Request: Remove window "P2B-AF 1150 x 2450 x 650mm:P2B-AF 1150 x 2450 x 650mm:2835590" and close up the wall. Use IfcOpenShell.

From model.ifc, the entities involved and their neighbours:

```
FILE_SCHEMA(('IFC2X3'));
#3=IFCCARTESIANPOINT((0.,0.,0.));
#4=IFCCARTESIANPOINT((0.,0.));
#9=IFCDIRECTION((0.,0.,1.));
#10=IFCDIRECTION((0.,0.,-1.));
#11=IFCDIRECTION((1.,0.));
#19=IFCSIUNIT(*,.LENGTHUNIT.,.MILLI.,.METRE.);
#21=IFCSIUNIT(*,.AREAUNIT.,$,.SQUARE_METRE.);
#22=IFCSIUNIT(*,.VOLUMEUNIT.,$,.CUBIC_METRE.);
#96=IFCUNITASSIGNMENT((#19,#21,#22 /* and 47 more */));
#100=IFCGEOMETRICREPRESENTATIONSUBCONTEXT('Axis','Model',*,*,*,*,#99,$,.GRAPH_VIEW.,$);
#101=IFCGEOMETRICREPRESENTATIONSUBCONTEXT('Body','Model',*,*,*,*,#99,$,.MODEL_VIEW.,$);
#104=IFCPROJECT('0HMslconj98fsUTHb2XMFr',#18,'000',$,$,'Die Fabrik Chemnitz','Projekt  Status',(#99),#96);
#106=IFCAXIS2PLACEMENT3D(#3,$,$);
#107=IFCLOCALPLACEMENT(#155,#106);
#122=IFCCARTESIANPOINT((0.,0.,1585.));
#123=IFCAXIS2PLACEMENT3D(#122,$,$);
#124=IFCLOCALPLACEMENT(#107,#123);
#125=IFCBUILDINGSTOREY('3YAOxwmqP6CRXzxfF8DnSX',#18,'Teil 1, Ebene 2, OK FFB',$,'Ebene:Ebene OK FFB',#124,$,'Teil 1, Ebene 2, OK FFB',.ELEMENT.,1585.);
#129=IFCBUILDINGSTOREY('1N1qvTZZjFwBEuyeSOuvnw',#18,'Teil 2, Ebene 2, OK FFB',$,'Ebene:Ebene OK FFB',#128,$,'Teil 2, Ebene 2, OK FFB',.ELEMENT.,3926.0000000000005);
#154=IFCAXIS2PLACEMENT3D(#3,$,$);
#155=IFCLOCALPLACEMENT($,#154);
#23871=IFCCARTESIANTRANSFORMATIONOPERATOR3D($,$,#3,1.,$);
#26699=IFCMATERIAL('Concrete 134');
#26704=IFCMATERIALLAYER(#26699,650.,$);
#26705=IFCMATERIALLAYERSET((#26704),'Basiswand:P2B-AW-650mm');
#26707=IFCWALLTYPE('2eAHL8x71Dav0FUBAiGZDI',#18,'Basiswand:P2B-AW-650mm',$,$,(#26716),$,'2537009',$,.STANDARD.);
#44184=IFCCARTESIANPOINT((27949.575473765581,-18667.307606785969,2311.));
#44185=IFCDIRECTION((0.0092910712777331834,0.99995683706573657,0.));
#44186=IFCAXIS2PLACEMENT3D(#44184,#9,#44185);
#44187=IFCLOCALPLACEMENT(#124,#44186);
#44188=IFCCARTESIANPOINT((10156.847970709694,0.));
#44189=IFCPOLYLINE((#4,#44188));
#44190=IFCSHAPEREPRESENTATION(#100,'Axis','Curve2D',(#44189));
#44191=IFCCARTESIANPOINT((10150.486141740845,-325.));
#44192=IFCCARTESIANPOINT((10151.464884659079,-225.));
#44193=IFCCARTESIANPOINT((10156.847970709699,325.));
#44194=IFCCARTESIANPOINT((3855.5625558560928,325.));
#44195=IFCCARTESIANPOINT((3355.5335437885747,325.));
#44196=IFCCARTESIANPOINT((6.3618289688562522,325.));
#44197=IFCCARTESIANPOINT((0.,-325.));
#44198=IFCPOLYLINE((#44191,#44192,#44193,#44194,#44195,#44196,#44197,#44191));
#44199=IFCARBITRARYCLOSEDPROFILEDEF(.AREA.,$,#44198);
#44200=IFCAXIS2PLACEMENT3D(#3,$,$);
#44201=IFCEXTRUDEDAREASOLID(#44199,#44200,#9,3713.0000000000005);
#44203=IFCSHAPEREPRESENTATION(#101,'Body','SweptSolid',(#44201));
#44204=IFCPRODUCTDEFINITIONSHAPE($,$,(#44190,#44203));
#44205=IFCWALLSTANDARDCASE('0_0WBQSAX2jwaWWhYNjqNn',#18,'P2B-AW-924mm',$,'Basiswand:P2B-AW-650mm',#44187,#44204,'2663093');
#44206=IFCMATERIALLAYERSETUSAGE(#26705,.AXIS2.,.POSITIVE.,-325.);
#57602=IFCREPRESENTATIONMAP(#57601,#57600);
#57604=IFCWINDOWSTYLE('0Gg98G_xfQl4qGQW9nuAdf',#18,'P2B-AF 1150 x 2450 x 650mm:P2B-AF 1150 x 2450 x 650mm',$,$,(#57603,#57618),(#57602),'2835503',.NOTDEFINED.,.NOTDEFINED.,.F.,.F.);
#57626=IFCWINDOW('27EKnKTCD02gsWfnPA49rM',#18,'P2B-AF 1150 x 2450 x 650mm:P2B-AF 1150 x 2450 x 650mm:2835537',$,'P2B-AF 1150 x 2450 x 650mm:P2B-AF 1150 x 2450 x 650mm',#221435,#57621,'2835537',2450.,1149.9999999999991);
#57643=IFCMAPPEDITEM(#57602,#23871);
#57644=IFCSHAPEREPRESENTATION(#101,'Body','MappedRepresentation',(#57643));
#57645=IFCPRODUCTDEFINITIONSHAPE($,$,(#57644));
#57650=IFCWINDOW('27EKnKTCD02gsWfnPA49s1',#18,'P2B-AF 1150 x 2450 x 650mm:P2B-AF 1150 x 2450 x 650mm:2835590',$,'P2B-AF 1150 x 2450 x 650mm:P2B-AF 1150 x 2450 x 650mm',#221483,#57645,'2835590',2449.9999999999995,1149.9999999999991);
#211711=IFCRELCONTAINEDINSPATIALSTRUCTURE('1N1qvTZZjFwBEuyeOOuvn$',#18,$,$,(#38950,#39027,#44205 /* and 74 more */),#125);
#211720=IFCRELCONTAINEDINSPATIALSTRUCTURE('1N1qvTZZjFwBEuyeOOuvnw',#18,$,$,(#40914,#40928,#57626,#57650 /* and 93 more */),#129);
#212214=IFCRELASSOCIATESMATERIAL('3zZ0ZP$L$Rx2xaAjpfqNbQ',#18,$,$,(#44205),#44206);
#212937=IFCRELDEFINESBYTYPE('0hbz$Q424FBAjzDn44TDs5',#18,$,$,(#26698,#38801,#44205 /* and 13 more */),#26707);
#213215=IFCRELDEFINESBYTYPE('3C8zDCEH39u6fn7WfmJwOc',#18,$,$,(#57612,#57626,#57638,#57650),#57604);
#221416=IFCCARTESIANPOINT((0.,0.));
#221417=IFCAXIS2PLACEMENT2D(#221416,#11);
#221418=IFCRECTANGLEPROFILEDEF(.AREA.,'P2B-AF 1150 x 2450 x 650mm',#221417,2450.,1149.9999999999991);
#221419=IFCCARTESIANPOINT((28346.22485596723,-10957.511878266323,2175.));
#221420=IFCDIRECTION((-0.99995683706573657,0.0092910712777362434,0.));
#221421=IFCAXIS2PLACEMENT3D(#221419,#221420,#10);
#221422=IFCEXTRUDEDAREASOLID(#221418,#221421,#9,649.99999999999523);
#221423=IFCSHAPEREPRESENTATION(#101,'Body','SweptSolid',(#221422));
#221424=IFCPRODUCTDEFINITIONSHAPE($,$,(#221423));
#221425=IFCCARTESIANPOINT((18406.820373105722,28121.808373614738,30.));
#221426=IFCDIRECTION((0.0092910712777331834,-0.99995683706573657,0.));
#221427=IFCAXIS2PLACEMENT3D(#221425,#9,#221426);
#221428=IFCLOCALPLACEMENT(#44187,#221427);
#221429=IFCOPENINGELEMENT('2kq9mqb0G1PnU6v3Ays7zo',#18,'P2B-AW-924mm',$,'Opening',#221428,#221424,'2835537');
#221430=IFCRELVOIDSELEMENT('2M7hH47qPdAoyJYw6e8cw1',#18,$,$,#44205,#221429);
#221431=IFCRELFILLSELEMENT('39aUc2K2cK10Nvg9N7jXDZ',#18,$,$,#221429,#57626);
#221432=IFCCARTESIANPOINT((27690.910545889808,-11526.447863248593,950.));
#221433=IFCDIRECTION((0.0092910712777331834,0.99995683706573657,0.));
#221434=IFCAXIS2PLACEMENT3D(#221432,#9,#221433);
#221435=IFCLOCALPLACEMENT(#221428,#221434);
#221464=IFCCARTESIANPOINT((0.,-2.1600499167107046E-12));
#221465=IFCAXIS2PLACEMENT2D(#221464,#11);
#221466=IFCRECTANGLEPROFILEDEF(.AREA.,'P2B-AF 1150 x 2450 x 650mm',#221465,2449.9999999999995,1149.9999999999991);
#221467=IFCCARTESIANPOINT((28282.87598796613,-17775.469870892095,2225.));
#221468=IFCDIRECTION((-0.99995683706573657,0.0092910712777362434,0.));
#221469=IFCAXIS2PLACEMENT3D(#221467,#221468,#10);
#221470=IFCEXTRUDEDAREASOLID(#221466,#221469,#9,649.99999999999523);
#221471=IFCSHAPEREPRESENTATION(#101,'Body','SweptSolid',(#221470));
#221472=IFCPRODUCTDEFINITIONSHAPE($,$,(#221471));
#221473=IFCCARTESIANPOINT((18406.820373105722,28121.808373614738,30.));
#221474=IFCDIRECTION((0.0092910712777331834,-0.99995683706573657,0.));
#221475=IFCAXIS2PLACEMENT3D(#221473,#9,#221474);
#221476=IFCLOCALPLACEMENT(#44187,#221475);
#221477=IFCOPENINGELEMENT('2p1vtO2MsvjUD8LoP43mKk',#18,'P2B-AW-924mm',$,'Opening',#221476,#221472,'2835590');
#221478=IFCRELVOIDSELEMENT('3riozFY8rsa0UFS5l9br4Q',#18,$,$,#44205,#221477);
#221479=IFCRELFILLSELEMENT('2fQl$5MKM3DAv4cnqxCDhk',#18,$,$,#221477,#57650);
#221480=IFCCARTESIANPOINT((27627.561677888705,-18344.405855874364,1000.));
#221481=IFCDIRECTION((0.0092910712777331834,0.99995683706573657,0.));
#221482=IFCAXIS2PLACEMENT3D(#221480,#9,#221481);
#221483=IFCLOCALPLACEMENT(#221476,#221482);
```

```python
import ifcopenshell
import ifcopenshell.api.feature
import ifcopenshell.api.root
import ifcopenshell.geom
import ifcopenshell.util.shape

model = ifcopenshell.open("model.ifc")
settings = ifcopenshell.geom.settings()


def volume(element):
    """Net volume in cubic metres, openings subtracted."""
    shape = ifcopenshell.geom.create_shape(settings, element)
    return ifcopenshell.util.shape.get_volume(shape.geometry)


window = model.by_guid("27EKnKTCD02gsWfnPA49s1")
opening = window.FillsVoids[0].RelatingOpeningElement
wall = opening.VoidsElements[0].RelatingBuildingElement
before = volume(wall)

ifcopenshell.api.root.remove_product(model, product=window)
ifcopenshell.api.feature.remove_feature(model, feature=opening)

after = volume(wall)

print(f"wall volume {before:.3f} -> {after:.3f} m3")

model.write("model_rev.ifc")
```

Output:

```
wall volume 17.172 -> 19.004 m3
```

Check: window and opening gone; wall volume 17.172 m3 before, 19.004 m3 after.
